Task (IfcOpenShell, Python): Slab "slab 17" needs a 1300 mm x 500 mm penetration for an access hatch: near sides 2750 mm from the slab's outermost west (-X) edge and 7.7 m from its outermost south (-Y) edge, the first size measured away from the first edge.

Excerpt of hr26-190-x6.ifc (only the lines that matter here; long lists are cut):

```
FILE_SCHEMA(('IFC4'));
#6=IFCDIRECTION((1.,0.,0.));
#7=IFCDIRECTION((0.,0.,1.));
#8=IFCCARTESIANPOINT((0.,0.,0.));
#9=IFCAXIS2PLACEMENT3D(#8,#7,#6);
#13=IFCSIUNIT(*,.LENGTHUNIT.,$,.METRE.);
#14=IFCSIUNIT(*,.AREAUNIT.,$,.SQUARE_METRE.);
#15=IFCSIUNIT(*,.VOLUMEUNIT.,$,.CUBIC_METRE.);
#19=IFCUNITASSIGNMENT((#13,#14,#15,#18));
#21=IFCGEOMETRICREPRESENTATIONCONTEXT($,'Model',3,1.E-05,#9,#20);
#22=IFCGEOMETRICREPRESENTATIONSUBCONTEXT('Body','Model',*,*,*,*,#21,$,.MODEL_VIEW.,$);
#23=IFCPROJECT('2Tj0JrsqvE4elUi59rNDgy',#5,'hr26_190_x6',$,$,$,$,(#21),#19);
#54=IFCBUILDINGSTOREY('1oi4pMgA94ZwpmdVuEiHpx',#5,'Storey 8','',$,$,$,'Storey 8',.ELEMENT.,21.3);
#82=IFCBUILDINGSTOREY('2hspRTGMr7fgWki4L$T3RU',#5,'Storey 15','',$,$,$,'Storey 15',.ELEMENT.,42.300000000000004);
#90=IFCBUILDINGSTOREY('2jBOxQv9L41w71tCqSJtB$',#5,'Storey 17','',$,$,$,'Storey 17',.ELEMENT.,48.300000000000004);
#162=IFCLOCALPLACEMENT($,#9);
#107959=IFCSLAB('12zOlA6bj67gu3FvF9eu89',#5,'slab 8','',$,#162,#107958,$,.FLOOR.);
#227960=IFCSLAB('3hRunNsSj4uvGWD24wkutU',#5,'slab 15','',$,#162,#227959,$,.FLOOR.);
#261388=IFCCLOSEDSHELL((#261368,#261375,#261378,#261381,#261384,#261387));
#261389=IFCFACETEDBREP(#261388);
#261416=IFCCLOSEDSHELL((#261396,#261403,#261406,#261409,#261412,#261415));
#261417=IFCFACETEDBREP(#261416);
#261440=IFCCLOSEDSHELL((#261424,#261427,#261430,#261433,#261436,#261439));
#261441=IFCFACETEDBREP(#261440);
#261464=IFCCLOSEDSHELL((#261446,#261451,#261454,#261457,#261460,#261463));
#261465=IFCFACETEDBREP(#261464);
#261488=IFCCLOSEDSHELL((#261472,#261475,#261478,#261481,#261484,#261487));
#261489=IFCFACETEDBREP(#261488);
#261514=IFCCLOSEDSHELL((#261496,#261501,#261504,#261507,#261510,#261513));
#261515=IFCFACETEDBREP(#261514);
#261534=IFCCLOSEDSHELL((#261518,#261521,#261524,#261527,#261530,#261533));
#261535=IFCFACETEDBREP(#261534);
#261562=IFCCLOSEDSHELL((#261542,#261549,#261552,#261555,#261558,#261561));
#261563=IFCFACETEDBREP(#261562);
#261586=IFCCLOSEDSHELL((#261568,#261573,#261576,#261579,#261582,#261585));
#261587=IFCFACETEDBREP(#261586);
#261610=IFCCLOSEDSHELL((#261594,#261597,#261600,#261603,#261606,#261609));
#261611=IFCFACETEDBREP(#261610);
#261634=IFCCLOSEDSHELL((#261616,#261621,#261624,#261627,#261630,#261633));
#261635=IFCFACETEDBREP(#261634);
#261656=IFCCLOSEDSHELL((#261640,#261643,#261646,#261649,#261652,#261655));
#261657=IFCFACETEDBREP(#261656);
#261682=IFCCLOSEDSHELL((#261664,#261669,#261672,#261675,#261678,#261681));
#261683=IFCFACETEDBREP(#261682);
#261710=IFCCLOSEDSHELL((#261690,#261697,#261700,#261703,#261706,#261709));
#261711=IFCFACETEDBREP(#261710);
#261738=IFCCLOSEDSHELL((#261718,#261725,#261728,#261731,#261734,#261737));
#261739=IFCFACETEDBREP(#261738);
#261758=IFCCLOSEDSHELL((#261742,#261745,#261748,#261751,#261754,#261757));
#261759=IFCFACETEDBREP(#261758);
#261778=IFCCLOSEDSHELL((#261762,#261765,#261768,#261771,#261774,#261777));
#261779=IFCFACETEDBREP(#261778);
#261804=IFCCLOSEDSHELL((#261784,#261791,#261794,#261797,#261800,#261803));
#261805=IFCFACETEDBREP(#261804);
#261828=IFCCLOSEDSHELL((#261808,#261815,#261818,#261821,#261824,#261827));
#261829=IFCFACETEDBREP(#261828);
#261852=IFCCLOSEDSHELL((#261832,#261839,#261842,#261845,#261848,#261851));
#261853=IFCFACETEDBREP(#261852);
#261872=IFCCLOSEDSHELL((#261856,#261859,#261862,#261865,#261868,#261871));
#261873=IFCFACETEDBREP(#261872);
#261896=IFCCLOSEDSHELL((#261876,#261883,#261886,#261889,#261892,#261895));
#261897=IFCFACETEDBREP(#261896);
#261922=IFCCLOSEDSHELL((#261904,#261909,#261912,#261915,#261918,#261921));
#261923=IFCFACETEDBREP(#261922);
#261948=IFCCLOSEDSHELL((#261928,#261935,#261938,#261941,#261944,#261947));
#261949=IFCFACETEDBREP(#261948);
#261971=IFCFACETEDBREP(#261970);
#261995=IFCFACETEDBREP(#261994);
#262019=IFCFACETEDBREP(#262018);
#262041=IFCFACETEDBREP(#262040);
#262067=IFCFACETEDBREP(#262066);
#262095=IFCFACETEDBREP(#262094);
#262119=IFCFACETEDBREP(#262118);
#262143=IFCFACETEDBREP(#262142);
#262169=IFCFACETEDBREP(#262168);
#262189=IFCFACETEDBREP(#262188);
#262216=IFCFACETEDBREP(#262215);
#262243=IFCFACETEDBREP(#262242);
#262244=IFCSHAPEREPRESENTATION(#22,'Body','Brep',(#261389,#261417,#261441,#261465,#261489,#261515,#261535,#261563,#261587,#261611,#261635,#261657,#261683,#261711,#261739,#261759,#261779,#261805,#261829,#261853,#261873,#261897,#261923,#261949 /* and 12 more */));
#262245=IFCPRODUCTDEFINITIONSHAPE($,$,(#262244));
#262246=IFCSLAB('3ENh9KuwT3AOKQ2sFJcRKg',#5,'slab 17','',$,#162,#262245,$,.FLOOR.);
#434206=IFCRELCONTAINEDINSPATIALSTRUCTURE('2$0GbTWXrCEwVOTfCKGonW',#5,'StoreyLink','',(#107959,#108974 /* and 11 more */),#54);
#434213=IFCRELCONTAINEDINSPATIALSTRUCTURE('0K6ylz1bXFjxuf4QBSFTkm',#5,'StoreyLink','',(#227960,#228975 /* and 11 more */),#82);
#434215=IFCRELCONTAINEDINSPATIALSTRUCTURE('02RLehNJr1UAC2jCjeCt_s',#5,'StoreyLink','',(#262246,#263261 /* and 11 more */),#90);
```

```python
import numpy as np
import ifcopenshell
import ifcopenshell.api.feature
import ifcopenshell.api.geometry
import ifcopenshell.api.root
import ifcopenshell.geom
import ifcopenshell.util.placement
import ifcopenshell.util.representation
import ifcopenshell.util.shape
import ifcopenshell.util.unit

model = ifcopenshell.open("hr26-190-x6.ifc")
unit_scale = ifcopenshell.util.unit.calculate_unit_scale(model)
settings = ifcopenshell.geom.settings()


def volume(element):
    """Net volume in cubic metres, openings subtracted."""
    shape = ifcopenshell.geom.create_shape(settings, element)
    return ifcopenshell.util.shape.get_volume(shape.geometry)


slab = model.by_guid("3ENh9KuwT3AOKQ2sFJcRKg")
before = volume(slab)

# Extent in the slab's own axes, in metres. The edges named are its -X and -Y sides.
slab_shape = ifcopenshell.geom.create_shape(settings, slab)
vertices = ifcopenshell.util.shape.get_vertices(slab_shape.geometry)
x_min, y_min, bottom = vertices.min(axis=0)
top = vertices[:, 2].max()

opening = ifcopenshell.api.root.create_entity(model, ifc_class="IfcOpeningElement", name="Access hatch opening", predefined_type="OPENING")
context = ifcopenshell.util.representation.get_context(model, "Model", "Body", "MODEL_VIEW")
width, depth = 1.3, 0.5
outline = [(0.0, 0.0), (width, 0.0), (width, depth), (0.0, depth), (0.0, 0.0)]
# Overshoot both faces by 50 mm so the cut is clean.
shape = ifcopenshell.api.geometry.add_slab_representation(
    model, context=context, depth=top - bottom + 0.1, polyline=outline
)
ifcopenshell.api.geometry.assign_representation(model, product=opening, representation=shape)

matrix = ifcopenshell.util.placement.get_local_placement(slab.ObjectPlacement)
matrix[:, 3] = matrix @ np.append(np.array([x_min + 2.75, y_min + 7.7, bottom - 0.05]) / unit_scale, 1.0)
ifcopenshell.api.geometry.edit_object_placement(model, product=opening, matrix=matrix, is_si=False)
ifcopenshell.api.feature.add_feature(model, feature=opening, element=slab)

after = volume(slab)

print(f"slab volume {before:.3f} -> {after:.3f} m3")

model.write("hr26-190-x6_updated.ifc")
```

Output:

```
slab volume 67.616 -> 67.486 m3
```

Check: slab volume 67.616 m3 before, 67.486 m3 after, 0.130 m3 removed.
